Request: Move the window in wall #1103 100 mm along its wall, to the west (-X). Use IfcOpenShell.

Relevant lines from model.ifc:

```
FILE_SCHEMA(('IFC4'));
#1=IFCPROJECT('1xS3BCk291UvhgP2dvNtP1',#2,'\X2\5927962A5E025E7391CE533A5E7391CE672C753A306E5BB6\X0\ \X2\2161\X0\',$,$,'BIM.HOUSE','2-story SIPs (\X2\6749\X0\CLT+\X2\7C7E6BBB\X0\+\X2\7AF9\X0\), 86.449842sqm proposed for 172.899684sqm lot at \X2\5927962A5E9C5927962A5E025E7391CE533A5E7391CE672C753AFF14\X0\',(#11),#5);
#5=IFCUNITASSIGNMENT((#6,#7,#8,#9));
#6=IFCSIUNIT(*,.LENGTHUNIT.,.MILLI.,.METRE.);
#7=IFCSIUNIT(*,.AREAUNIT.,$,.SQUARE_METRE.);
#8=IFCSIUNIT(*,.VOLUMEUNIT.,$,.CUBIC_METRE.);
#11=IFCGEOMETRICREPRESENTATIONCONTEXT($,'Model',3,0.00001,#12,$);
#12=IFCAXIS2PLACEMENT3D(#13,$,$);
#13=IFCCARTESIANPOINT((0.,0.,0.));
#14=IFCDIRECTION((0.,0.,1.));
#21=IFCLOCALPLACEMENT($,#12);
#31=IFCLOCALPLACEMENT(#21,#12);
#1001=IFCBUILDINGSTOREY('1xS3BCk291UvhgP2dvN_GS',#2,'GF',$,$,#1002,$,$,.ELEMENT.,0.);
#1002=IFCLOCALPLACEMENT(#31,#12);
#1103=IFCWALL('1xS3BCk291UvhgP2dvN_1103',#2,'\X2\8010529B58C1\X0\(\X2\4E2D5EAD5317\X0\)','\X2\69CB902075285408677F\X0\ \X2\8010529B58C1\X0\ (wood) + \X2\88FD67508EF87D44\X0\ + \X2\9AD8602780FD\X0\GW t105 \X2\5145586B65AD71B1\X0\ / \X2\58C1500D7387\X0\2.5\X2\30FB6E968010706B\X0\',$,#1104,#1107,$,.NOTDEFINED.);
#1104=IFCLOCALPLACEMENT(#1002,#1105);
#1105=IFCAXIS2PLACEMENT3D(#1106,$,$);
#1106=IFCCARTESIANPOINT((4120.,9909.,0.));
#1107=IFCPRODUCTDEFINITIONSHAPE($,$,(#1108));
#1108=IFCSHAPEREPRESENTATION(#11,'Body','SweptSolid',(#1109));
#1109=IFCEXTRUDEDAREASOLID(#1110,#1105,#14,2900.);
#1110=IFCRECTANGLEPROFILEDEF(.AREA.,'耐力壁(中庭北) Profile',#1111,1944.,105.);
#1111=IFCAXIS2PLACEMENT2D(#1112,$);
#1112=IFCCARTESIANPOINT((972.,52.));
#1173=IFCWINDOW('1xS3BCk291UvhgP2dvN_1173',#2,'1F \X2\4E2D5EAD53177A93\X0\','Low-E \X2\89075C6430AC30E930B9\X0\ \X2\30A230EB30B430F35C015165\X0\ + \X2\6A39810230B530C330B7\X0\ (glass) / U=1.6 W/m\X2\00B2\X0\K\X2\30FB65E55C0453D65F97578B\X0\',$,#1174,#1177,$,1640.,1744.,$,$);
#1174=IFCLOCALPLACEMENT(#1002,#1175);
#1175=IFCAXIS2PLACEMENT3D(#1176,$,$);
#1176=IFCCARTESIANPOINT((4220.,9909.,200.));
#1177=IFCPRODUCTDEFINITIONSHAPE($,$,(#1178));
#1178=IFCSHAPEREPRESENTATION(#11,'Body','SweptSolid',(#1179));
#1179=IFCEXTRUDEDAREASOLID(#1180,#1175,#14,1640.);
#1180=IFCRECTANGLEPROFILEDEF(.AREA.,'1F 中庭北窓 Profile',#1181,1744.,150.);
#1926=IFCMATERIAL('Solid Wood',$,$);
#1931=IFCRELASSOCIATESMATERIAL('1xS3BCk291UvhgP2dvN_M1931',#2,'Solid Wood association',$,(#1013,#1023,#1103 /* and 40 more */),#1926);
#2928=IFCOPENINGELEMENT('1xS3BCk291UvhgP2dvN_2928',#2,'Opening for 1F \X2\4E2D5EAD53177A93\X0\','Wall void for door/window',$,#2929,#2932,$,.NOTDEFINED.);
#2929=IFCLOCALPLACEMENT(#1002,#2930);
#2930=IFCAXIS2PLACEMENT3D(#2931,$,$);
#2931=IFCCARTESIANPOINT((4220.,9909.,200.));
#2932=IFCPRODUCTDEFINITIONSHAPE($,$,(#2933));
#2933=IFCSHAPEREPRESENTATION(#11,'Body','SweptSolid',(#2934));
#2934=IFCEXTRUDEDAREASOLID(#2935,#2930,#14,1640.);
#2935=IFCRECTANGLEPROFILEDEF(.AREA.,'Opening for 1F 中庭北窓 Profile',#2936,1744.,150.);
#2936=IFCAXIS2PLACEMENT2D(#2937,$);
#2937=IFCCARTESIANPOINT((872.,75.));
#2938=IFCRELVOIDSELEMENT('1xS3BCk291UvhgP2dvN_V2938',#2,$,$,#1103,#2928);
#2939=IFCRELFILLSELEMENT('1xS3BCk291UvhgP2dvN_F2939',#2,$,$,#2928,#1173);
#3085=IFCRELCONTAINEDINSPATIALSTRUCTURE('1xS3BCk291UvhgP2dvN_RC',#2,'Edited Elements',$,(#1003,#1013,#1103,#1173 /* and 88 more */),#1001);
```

```python
import ifcopenshell
import ifcopenshell.api.geometry
import ifcopenshell.util.placement

model = ifcopenshell.open("model.ifc")

window = model.by_guid("1xS3BCk291UvhgP2dvN_1173")
opening = window.FillsVoids[0].RelatingOpeningElement
wall = opening.VoidsElements[0].RelatingBuildingElement

wall_matrix = ifcopenshell.util.placement.get_local_placement(wall.ObjectPlacement)
shift = wall_matrix[:3, 0] * -100.0
before = ifcopenshell.util.placement.get_local_placement(window.ObjectPlacement)[:3, 3].copy()

# The window is not placed relative to its opening, so move both.
for product in (opening, window):
    matrix = ifcopenshell.util.placement.get_local_placement(product.ObjectPlacement)
    matrix[:3, 3] += shift
    ifcopenshell.api.geometry.edit_object_placement(model, product=product, matrix=matrix, is_si=False)

after = ifcopenshell.util.placement.get_local_placement(window.ObjectPlacement)[:3, 3]
print("window moved by", (after - before).round(3) + 0.0)

model.write("model_edited.ifc")
```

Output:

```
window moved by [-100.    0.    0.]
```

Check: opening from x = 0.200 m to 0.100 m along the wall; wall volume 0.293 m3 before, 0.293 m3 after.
